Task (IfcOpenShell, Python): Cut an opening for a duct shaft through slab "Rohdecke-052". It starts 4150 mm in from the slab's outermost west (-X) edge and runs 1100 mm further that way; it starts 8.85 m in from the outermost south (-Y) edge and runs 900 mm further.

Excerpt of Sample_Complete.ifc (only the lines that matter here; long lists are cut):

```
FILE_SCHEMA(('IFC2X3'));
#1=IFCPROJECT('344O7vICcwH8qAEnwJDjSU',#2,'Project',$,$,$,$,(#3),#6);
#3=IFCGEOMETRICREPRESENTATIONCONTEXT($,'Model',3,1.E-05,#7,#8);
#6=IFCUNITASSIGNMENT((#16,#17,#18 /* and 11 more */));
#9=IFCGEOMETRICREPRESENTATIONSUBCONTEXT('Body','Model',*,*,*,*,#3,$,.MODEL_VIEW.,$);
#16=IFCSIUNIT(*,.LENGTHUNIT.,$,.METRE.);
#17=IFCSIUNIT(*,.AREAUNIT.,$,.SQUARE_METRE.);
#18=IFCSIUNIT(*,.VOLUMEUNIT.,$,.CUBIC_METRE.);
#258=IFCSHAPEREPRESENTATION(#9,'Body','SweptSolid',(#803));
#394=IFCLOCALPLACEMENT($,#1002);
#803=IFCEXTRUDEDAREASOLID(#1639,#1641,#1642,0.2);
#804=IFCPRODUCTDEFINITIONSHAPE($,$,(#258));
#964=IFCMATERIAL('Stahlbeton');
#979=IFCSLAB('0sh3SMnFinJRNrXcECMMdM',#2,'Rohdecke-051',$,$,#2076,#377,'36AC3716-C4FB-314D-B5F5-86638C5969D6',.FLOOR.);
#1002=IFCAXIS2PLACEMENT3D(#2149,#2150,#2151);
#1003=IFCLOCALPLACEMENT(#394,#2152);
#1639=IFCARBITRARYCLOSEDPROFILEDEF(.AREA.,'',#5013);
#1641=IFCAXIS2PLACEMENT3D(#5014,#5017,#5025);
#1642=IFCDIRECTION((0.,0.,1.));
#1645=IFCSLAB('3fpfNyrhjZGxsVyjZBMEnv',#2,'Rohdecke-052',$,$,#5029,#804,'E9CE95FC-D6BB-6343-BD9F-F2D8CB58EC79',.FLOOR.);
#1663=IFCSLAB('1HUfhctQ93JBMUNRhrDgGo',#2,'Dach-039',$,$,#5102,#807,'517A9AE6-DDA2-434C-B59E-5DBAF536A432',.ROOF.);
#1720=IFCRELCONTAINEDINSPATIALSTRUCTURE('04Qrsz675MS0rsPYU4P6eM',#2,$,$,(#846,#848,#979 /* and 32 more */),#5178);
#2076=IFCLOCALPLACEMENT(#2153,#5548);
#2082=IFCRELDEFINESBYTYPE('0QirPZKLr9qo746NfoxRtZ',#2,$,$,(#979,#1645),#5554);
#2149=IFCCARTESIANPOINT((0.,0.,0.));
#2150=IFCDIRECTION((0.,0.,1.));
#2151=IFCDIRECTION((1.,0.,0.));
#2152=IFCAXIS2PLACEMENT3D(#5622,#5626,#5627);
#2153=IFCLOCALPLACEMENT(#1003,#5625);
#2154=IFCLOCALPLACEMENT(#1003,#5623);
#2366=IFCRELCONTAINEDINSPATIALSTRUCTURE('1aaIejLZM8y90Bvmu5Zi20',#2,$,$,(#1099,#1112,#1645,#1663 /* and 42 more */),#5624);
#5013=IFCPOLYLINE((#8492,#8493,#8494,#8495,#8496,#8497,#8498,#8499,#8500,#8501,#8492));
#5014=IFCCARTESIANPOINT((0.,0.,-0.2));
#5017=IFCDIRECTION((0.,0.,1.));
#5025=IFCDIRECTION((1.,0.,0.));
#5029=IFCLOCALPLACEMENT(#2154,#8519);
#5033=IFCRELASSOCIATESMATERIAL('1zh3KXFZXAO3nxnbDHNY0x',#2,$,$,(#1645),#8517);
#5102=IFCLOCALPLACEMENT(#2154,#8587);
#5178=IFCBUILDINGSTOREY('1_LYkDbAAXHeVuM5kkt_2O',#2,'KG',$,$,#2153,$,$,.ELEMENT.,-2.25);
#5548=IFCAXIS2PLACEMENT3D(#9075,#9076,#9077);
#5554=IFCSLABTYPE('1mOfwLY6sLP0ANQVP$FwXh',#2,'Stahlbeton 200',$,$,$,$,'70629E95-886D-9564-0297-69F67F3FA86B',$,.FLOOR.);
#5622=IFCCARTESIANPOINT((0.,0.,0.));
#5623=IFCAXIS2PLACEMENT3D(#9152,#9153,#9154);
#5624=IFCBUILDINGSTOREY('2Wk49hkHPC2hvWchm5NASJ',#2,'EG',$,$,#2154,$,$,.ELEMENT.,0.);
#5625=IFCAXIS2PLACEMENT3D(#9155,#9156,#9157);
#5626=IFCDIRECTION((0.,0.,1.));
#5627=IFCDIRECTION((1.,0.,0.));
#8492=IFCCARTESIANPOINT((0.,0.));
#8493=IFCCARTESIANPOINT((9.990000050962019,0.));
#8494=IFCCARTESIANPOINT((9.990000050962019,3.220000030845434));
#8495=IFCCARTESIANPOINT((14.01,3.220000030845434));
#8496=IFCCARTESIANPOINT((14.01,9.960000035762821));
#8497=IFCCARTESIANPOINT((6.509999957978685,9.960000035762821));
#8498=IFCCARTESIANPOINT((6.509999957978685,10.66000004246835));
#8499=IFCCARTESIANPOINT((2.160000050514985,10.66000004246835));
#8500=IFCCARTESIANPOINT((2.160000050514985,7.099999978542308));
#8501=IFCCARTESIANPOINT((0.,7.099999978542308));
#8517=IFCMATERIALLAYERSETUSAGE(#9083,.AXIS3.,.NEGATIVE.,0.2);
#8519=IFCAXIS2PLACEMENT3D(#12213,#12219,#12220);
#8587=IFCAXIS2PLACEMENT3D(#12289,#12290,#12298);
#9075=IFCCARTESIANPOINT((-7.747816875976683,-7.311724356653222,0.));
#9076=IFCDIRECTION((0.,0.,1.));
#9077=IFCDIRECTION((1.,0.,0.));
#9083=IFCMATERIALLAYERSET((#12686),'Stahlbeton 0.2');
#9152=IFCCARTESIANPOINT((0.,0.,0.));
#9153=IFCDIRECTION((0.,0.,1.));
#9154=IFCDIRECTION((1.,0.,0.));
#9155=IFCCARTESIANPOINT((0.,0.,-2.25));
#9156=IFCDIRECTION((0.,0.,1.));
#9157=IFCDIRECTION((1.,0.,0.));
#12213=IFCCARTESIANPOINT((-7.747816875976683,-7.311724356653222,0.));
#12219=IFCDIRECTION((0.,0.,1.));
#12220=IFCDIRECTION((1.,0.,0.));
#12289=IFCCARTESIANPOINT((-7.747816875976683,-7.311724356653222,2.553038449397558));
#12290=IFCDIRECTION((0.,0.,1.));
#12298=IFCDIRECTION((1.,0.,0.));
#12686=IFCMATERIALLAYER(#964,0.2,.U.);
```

```python
import numpy as np
import ifcopenshell
import ifcopenshell.api.feature
import ifcopenshell.api.geometry
import ifcopenshell.api.root
import ifcopenshell.geom
import ifcopenshell.util.placement
import ifcopenshell.util.representation
import ifcopenshell.util.shape
import ifcopenshell.util.unit

model = ifcopenshell.open("Sample_Complete.ifc")
unit_scale = ifcopenshell.util.unit.calculate_unit_scale(model)
settings = ifcopenshell.geom.settings()


def volume(element):
    """Net volume in cubic metres, openings subtracted."""
    shape = ifcopenshell.geom.create_shape(settings, element)
    return ifcopenshell.util.shape.get_volume(shape.geometry)


slab = model.by_id(1645)
before = volume(slab)

# Extent in the slab's own axes, in metres. The edges named are its -X and -Y sides.
slab_shape = ifcopenshell.geom.create_shape(settings, slab)
vertices = ifcopenshell.util.shape.get_vertices(slab_shape.geometry)
x_min, y_min, bottom = vertices.min(axis=0)
top = vertices[:, 2].max()

opening = ifcopenshell.api.root.create_entity(model, ifc_class="IfcOpeningElement", name="Duct shaft opening")
context = ifcopenshell.util.representation.get_context(model, "Model", "Body", "MODEL_VIEW")
width, depth = 1.1, 0.9
outline = [(0.0, 0.0), (width, 0.0), (width, depth), (0.0, depth), (0.0, 0.0)]
# Overshoot both faces by 50 mm so the cut is clean.
shape = ifcopenshell.api.geometry.add_slab_representation(
    model, context=context, depth=top - bottom + 0.1, polyline=outline
)
ifcopenshell.api.geometry.assign_representation(model, product=opening, representation=shape)

matrix = ifcopenshell.util.placement.get_local_placement(slab.ObjectPlacement)
matrix[:, 3] = matrix @ np.append(np.array([x_min + 4.15, y_min + 8.85, bottom - 0.05]) / unit_scale, 1.0)
ifcopenshell.api.geometry.edit_object_placement(model, product=opening, matrix=matrix, is_si=False)
ifcopenshell.api.feature.add_feature(model, feature=opening, element=slab)

after = volume(slab)

print(f"slab volume {before:.3f} -> {after:.3f} m3")

model.write("Sample_Complete_edited.ifc")
```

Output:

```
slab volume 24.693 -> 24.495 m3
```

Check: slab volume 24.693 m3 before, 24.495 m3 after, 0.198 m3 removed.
